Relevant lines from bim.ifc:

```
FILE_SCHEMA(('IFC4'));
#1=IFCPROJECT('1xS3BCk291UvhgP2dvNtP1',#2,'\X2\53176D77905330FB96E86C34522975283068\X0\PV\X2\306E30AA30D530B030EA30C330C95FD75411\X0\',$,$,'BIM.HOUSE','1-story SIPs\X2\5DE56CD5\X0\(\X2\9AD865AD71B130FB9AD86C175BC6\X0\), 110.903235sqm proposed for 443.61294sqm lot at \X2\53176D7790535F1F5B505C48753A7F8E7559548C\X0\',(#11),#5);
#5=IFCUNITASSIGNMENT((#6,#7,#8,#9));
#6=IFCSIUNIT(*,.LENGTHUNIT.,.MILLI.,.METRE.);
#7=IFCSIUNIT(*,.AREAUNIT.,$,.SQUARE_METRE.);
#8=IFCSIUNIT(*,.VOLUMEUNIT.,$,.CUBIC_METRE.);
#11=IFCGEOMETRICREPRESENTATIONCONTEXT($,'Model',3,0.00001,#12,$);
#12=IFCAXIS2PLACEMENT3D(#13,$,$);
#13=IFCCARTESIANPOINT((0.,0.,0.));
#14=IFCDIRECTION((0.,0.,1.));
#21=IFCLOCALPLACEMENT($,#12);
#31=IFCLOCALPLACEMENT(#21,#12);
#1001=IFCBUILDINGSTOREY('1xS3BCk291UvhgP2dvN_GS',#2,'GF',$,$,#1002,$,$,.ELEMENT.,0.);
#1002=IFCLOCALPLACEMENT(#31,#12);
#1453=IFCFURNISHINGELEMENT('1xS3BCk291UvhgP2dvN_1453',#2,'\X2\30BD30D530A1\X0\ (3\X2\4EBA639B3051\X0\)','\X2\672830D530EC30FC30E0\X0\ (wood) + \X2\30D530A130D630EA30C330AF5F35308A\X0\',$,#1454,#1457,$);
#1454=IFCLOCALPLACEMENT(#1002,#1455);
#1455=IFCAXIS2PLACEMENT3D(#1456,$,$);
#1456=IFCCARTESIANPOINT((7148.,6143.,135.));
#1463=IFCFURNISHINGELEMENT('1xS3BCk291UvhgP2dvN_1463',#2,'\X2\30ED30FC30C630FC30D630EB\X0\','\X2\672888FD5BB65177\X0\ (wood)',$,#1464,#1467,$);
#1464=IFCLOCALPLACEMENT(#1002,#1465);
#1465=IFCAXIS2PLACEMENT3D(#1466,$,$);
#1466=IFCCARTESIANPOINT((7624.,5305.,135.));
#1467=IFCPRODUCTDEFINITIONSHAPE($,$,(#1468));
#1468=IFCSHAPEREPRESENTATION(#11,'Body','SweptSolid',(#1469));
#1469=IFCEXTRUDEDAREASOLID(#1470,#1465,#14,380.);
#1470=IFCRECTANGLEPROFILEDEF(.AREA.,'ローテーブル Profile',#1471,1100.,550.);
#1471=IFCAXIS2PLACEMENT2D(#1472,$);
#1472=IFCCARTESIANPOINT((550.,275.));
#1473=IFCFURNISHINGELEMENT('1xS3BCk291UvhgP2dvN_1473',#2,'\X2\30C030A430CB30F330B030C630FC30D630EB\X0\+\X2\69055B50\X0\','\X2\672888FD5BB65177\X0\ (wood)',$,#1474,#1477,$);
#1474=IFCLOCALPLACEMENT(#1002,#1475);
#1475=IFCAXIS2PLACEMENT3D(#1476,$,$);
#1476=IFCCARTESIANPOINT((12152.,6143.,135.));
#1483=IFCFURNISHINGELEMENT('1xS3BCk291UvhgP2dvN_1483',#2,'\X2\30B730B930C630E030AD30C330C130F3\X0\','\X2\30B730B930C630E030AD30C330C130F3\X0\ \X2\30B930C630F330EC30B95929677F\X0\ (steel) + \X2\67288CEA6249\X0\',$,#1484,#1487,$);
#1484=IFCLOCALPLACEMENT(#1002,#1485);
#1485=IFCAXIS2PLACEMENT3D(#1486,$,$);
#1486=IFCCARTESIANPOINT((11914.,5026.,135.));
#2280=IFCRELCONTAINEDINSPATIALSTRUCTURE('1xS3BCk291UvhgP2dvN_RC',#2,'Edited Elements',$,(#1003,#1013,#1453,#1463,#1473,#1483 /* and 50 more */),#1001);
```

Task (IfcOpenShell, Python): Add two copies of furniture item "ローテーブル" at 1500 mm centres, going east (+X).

```python
import numpy as np
import ifcopenshell
import ifcopenshell.api.geometry
import ifcopenshell.api.root
import ifcopenshell.util.element
import ifcopenshell.util.placement
import ifcopenshell.util.unit

model = ifcopenshell.open("bim.ifc")
unit_scale = ifcopenshell.util.unit.calculate_unit_scale(model)


def reuse_history(source, copy):
    """copy_class also copies each property set's owner history, people and application; keep the originals."""
    for rel in copy.IsDefinedBy:
        if rel.is_a("IfcRelDefinesByProperties") and (history := rel.RelatingPropertyDefinition.OwnerHistory):
            rel.RelatingPropertyDefinition.OwnerHistory = source.OwnerHistory
            ifcopenshell.util.element.remove_deep2(model, history)


source = model.by_guid("1xS3BCk291UvhgP2dvN_1463")
base = ifcopenshell.util.placement.get_local_placement(source.ObjectPlacement)
step = np.array([1.0, 0.0, 0.0]) * 1.5 / unit_scale

for i in range(1, 3):
    copy = ifcopenshell.api.root.copy_class(model, product=source)
    copy.Representation = ifcopenshell.util.element.copy_deep(
        model, source.Representation, exclude=["IfcGeometricRepresentationContext", "IfcRepresentationMap"]
    )
    reuse_history(source, copy)
    matrix = base.copy()
    matrix[:3, 3] += i * step
    print("added at", matrix[:3, 3].round(3) + 0.0)
    ifcopenshell.api.geometry.edit_object_placement(model, product=copy, matrix=matrix, is_si=False)

model.write("bim_edited.ifc")
```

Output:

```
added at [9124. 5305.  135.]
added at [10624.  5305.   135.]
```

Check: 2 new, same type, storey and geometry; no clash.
